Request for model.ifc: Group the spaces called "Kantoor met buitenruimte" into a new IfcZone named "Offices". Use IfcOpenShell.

First a look at what the model holds.

```python
import ifcopenshell

model = ifcopenshell.open("model.ifc")
print(model.schema)
seen = {}
for space in model.by_type("IfcSpace"):
    seen[space.LongName] = seen.get(space.LongName, 0) + 1
for name, count in sorted(seen.items(), key=str):
    print(count, "x", name)
print("zones:", [z.Name for z in model.by_type("IfcZone")][:20])
```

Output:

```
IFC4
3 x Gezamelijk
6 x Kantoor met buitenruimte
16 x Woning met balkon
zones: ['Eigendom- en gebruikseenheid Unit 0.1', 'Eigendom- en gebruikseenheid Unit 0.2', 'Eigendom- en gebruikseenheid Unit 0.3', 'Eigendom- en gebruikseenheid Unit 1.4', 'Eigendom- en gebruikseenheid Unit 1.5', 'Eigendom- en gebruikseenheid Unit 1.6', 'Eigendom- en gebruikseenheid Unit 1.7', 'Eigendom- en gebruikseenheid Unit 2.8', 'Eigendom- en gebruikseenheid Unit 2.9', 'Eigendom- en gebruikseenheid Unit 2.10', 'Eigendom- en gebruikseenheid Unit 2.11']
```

```python
import ifcopenshell
import ifcopenshell.api.group
import ifcopenshell.api.root

model = ifcopenshell.open("model.ifc")

names = {"Kantoor met buitenruimte"}
spaces = [s for s in model.by_type("IfcSpace") if s.LongName in names]

zone = ifcopenshell.api.root.create_entity(model, ifc_class="IfcZone", name="Offices")
ifcopenshell.api.group.assign_group(model, products=spaces, group=zone)
print(len(spaces), "spaces in", zone.Name)

model.write("model_edited.ifc")
```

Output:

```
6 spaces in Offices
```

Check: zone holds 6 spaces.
